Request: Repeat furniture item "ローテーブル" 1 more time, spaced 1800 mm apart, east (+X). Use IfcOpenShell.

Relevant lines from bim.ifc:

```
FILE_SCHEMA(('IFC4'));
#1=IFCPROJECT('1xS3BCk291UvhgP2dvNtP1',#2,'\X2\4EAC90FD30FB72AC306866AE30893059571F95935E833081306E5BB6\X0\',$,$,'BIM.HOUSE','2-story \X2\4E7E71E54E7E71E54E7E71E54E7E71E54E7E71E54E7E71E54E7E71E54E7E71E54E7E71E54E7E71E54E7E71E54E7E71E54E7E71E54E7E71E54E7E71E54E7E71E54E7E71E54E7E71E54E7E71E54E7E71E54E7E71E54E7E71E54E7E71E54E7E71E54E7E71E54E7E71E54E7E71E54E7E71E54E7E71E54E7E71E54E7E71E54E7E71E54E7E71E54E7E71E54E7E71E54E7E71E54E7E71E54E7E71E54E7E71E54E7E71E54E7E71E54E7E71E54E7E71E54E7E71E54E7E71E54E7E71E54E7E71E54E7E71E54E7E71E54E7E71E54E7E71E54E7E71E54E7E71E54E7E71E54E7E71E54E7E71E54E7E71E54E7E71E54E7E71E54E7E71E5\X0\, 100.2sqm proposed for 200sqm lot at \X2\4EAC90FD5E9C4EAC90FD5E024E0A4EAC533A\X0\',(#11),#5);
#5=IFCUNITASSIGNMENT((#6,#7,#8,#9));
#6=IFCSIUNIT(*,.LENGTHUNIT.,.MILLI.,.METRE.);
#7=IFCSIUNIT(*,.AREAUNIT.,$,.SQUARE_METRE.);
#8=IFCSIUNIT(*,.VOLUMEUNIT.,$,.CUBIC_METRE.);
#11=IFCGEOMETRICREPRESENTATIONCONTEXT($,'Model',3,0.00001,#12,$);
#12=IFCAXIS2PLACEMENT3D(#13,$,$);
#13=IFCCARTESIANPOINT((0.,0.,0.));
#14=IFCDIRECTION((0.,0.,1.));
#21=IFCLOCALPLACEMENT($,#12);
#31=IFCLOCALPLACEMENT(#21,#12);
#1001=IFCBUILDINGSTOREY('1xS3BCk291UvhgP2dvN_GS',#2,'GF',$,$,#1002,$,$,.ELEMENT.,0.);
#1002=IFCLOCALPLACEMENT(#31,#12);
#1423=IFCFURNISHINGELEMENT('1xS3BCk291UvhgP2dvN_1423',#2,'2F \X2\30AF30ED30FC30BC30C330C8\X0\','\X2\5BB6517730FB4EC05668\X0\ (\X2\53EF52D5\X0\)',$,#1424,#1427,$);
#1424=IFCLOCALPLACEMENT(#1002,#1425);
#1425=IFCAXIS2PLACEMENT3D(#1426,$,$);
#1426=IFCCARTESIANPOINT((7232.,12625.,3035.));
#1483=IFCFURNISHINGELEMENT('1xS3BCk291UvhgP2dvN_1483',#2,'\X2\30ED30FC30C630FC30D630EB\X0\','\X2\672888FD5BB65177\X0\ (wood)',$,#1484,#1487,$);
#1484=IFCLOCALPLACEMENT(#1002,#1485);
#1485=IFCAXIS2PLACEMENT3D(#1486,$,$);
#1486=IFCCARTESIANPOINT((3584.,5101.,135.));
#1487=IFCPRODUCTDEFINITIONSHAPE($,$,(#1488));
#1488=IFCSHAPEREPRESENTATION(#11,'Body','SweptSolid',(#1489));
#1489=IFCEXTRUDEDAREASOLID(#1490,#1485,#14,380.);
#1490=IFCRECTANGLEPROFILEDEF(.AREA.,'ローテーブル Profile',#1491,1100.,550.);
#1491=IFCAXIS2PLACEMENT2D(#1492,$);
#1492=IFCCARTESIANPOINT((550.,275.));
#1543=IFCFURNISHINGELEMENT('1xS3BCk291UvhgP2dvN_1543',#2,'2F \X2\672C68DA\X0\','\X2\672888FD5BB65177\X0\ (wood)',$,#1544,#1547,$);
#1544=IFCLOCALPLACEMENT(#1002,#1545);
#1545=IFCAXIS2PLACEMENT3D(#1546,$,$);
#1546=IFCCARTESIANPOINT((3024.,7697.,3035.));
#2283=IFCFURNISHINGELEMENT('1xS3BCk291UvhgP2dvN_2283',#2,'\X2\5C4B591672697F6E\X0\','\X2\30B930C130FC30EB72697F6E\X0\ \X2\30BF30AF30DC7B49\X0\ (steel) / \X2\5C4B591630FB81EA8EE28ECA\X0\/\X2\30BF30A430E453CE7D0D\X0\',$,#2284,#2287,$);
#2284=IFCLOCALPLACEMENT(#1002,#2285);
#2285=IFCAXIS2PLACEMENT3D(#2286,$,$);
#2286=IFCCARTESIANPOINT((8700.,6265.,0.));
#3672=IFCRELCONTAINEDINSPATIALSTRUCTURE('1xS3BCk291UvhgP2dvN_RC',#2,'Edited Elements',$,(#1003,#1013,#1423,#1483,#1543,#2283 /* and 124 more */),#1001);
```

```python
import numpy as np
import ifcopenshell
import ifcopenshell.api.geometry
import ifcopenshell.api.root
import ifcopenshell.util.element
import ifcopenshell.util.placement
import ifcopenshell.util.unit

model = ifcopenshell.open("bim.ifc")
unit_scale = ifcopenshell.util.unit.calculate_unit_scale(model)


def reuse_history(source, copy):
    """copy_class also copies each property set's owner history, people and application; keep the originals."""
    for rel in copy.IsDefinedBy:
        if rel.is_a("IfcRelDefinesByProperties") and (history := rel.RelatingPropertyDefinition.OwnerHistory):
            rel.RelatingPropertyDefinition.OwnerHistory = source.OwnerHistory
            ifcopenshell.util.element.remove_deep2(model, history)


source = model.by_id(1483)
base = ifcopenshell.util.placement.get_local_placement(source.ObjectPlacement)
step = np.array([1.0, 0.0, 0.0]) * 1.8 / unit_scale

for i in range(1, 2):
    copy = ifcopenshell.api.root.copy_class(model, product=source)
    copy.Representation = ifcopenshell.util.element.copy_deep(
        model, source.Representation, exclude=["IfcGeometricRepresentationContext", "IfcRepresentationMap"]
    )
    reuse_history(source, copy)
    matrix = base.copy()
    matrix[:3, 3] += i * step
    print("added at", matrix[:3, 3].round(3) + 0.0)
    ifcopenshell.api.geometry.edit_object_placement(model, product=copy, matrix=matrix, is_si=False)

model.write("bim_rev.ifc")
```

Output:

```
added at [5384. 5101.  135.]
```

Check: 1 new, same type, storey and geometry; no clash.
